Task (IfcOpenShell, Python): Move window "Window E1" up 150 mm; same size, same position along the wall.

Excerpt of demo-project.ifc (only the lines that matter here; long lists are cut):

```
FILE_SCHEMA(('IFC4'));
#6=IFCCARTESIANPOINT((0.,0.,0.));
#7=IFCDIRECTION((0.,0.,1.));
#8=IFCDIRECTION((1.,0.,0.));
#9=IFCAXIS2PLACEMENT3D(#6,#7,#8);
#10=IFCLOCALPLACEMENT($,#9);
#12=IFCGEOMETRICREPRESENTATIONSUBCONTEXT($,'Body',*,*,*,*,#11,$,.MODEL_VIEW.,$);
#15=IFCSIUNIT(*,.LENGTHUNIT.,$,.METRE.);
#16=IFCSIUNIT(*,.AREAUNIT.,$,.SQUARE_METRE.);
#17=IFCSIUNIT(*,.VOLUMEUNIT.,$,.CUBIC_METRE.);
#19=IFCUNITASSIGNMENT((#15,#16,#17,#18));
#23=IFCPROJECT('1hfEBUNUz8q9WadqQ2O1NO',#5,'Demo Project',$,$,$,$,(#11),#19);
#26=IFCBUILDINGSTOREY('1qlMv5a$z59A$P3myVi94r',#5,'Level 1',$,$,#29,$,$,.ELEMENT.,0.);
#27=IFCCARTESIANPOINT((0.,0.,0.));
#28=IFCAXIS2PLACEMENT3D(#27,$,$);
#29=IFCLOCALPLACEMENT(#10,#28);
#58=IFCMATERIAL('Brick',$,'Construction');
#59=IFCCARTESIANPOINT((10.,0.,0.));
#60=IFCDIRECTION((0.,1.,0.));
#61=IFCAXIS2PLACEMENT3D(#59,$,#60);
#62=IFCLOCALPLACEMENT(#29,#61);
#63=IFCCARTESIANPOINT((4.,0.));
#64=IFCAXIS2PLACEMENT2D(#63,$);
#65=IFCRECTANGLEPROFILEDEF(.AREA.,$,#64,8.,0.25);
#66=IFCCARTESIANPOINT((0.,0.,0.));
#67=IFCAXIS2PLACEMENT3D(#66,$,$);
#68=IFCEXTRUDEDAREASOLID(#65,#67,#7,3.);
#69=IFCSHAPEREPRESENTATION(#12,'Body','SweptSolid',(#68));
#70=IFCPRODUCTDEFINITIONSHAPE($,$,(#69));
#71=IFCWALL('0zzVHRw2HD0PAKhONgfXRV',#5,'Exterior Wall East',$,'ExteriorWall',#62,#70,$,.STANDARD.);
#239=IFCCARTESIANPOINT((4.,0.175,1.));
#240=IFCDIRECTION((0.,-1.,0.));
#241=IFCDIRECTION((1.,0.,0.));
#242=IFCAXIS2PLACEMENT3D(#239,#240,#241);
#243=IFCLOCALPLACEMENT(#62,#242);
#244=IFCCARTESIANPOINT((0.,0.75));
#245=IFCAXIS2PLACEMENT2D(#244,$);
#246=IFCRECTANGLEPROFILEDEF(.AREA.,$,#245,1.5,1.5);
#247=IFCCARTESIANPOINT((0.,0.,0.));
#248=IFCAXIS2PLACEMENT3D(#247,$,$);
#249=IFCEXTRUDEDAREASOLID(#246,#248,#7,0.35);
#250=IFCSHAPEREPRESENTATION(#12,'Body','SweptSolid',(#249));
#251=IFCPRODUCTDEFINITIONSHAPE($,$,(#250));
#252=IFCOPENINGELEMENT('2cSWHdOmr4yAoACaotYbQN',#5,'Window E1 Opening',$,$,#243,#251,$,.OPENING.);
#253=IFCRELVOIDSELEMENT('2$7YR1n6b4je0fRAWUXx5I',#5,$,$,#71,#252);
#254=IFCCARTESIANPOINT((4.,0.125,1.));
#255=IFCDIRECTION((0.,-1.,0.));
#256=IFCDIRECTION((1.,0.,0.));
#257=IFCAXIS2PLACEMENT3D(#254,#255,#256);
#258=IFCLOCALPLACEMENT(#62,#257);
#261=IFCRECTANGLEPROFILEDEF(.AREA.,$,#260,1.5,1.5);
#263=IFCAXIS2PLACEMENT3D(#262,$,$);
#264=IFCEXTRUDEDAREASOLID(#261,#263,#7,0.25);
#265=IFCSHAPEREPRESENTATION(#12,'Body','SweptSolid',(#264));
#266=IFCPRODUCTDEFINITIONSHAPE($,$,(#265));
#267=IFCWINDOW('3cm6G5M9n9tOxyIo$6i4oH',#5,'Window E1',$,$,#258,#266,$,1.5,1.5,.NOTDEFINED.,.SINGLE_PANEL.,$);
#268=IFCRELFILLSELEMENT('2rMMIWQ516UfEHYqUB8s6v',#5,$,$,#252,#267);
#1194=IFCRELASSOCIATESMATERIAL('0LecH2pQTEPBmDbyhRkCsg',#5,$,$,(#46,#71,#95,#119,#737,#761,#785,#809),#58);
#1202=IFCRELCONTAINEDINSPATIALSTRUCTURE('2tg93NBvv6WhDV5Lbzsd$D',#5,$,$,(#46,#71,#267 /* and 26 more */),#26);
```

```python
import numpy as np
import ifcopenshell
import ifcopenshell.api.geometry
import ifcopenshell.util.placement
import ifcopenshell.util.unit

model = ifcopenshell.open("demo-project.ifc")
unit_scale = ifcopenshell.util.unit.calculate_unit_scale(model)

window = model.by_guid("3cm6G5M9n9tOxyIo$6i4oH")
opening = window.FillsVoids[0].RelatingOpeningElement
dz = 0.15

shift = np.array([0.0, 0.0, dz])
# The window is not placed relative to its opening, so move both.
for product in (opening, window):
    matrix = ifcopenshell.util.placement.get_local_placement(product.ObjectPlacement)
    matrix[:3, 3] += shift
    ifcopenshell.api.geometry.edit_object_placement(model, product=product, matrix=matrix, is_si=False)

print(f"moved by {dz * unit_scale:+.3f} m")

model.write("demo-project_updated.ifc")
```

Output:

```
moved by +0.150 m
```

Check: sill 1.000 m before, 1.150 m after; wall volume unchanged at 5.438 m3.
